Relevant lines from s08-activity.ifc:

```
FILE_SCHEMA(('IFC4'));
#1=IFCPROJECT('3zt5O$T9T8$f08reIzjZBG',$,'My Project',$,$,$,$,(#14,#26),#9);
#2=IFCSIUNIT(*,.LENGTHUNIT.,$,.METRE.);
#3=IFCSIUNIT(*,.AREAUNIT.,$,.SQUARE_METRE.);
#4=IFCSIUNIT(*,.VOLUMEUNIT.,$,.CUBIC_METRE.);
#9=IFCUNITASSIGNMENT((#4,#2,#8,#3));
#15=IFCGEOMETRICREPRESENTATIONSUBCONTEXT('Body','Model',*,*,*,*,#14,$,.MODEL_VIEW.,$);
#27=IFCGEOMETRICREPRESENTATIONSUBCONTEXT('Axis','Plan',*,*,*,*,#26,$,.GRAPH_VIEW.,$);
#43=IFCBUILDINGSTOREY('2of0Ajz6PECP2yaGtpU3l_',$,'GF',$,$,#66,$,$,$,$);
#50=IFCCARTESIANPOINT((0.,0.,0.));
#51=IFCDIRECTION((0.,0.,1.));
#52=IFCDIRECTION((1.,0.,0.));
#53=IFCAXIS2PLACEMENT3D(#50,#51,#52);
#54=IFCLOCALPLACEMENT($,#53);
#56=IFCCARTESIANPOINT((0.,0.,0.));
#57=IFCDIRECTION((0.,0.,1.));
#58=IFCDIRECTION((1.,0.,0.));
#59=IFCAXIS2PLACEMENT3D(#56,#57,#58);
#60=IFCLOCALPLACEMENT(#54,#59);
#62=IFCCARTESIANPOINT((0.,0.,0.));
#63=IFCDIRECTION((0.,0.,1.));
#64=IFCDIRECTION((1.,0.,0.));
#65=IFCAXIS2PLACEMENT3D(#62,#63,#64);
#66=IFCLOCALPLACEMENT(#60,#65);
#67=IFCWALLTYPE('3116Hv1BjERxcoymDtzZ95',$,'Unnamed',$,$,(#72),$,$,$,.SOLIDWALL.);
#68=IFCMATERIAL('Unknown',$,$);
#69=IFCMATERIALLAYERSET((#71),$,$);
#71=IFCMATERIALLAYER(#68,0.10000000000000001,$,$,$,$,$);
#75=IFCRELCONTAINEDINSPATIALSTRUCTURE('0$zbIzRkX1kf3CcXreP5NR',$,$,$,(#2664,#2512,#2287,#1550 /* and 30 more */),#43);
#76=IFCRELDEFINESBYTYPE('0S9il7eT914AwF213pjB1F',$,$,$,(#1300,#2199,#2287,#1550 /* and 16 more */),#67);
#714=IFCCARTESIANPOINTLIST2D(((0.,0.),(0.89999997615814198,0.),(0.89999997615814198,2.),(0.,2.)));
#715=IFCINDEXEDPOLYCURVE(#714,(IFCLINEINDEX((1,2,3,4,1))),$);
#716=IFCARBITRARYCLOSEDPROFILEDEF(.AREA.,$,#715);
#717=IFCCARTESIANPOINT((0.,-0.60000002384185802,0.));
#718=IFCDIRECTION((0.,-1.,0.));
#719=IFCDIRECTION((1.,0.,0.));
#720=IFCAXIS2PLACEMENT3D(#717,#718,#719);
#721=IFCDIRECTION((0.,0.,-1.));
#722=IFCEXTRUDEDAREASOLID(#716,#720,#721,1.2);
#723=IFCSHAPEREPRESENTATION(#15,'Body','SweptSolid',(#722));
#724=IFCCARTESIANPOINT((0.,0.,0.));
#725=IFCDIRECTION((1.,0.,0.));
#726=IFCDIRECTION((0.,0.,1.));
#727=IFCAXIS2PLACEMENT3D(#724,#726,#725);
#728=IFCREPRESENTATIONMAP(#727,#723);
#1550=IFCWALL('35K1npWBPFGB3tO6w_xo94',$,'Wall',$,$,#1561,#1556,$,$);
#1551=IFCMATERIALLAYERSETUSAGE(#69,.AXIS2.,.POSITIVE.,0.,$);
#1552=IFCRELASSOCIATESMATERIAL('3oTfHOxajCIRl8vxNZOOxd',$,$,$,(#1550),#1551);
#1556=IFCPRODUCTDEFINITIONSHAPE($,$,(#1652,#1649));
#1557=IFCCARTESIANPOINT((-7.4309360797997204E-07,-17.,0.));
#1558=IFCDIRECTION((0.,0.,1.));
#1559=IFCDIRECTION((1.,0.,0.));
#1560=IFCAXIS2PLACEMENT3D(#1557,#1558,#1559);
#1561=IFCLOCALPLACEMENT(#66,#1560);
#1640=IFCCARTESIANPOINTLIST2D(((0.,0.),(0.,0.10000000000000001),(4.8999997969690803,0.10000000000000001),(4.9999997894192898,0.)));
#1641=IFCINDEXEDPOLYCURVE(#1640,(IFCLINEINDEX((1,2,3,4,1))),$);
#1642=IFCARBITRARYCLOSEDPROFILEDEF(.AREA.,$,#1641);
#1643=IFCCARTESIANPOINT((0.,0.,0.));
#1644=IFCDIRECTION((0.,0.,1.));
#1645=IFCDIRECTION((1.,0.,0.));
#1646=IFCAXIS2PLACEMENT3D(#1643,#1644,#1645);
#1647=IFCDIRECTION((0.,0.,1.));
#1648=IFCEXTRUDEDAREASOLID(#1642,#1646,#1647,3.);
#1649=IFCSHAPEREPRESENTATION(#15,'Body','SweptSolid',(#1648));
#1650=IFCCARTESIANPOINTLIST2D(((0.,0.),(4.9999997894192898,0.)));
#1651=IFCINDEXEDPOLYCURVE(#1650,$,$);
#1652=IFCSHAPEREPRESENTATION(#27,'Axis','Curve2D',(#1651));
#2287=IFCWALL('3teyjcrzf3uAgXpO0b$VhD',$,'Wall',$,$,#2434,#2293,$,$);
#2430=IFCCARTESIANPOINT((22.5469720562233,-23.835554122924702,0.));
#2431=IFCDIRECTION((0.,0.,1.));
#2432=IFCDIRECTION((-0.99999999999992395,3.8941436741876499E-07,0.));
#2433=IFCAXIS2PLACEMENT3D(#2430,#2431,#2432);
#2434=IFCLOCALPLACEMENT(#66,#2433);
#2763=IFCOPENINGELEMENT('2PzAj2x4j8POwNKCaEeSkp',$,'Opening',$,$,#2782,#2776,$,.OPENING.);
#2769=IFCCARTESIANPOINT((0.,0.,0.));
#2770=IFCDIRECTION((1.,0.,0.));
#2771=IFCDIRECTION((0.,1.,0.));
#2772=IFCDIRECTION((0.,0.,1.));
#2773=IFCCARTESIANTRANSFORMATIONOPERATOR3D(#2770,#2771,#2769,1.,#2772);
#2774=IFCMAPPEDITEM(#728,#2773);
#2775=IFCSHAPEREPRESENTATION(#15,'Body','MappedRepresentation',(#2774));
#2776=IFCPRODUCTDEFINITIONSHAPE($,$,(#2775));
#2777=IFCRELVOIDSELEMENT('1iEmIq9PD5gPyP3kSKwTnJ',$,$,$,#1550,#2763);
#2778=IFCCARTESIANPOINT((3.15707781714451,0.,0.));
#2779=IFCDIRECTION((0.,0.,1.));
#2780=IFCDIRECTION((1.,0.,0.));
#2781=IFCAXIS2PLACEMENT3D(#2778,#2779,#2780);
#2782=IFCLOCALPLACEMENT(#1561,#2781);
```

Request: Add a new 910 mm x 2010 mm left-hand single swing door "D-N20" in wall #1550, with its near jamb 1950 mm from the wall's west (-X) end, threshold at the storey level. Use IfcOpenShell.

```python
import numpy as np
import ifcopenshell
import ifcopenshell.api.feature
import ifcopenshell.api.geometry
import ifcopenshell.api.root
import ifcopenshell.api.spatial
import ifcopenshell.geom
import ifcopenshell.util.element
import ifcopenshell.util.placement
import ifcopenshell.util.representation
import ifcopenshell.util.shape
import ifcopenshell.util.unit

model = ifcopenshell.open("s08-activity.ifc")
unit_scale = ifcopenshell.util.unit.calculate_unit_scale(model)
settings = ifcopenshell.geom.settings()


def volume(element):
    """Net volume in cubic metres, openings subtracted."""
    shape = ifcopenshell.geom.create_shape(settings, element)
    return ifcopenshell.util.shape.get_volume(shape.geometry)


wall = model.by_id(1550)
storey = ifcopenshell.util.element.get_container(wall, ifc_class="IfcBuildingStorey")
context = ifcopenshell.util.representation.get_context(model, "Model", "Body", "MODEL_VIEW")
before = volume(wall)

width, height, from_end, sill = 0.91, 2.01, 1.95, 0.0  # metres

# The wall runs along its own X axis, and the end named is its -X end.
wall_shape = ifcopenshell.geom.create_shape(settings, wall)
x, y, z = ifcopenshell.util.shape.get_vertices(wall_shape.geometry).T
start = x.min() + from_end
face, thickness = float(y.min()), float(y.max() - y.min())
wall_matrix = ifcopenshell.util.placement.get_local_placement(wall.ObjectPlacement)
level = ifcopenshell.util.placement.get_local_placement(storey.ObjectPlacement)[2, 3]


def in_wall(x, y):
    """Placement at x, y metres in the wall's axes, at sill height."""
    matrix = wall_matrix.copy()
    matrix[:, 3] = wall_matrix @ np.array([x / unit_scale, y / unit_scale, 0.0, 1.0])
    matrix[2, 3] = level + sill / unit_scale
    return matrix


# Opening: a box that overshoots both wall faces by 50 mm.
opening = ifcopenshell.api.root.create_entity(model, ifc_class="IfcOpeningElement", predefined_type="OPENING")
box = ifcopenshell.api.geometry.add_wall_representation(
    model, context=context, length=width, height=height, thickness=thickness + 0.1
)
ifcopenshell.api.geometry.assign_representation(model, product=opening, representation=box)
ifcopenshell.api.geometry.edit_object_placement(model, product=opening, matrix=in_wall(start, face - 0.05), is_si=False)
ifcopenshell.api.feature.add_feature(model, feature=opening, element=wall)

door = ifcopenshell.api.root.create_entity(model, ifc_class="IfcDoor", name="D-N20", predefined_type="DOOR")
door.OverallWidth, door.OverallHeight = width / unit_scale, height / unit_scale
door.OperationType = "SINGLE_SWING_LEFT"
body = ifcopenshell.api.geometry.add_door_representation(
    model,
    context=context,
    overall_width=door.OverallWidth,
    overall_height=door.OverallHeight,
    operation_type="SINGLE_SWING_LEFT",
    lining_properties={"LiningDepth": thickness / unit_scale, "ThresholdDepth": thickness / unit_scale},
)
ifcopenshell.api.geometry.assign_representation(model, product=door, representation=body)
ifcopenshell.api.spatial.assign_container(model, products=[door], relating_structure=storey)
ifcopenshell.api.feature.add_filling(model, opening=opening, element=door)

# The lining spans the wall, so the door starts at the wall face.
ifcopenshell.api.geometry.edit_object_placement(model, product=door, matrix=in_wall(start, face), is_si=False)

after = volume(wall)

print(f"wall volume {before:.3f} -> {after:.3f} m3")

model.write("s08-activity_updated.ifc")
```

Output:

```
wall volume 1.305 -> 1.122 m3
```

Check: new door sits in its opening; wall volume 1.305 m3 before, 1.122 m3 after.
